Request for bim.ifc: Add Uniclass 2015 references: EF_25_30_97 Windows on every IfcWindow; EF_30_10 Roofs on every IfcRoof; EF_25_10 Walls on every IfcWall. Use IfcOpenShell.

First a look at what the model holds.

```python
import ifcopenshell

model = ifcopenshell.open("bim.ifc")
print(model.schema)
print("classifications:", [c.Name for c in model.by_type("IfcClassification")])
for ifc_class in ("IfcDoor", "IfcRoof", "IfcStair", "IfcWall", "IfcWindow"):
    print(ifc_class, len(model.by_type(ifc_class)))
```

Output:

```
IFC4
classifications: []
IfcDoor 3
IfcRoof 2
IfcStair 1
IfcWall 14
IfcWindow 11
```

```python
import ifcopenshell
import ifcopenshell.api.classification

model = ifcopenshell.open("bim.ifc")

system = ifcopenshell.api.classification.add_classification(model, classification="Uniclass 2015")

codes = {
    "IfcWindow": ("EF_25_30_97", "Windows"),
    "IfcRoof": ("EF_30_10", "Roofs"),
    "IfcWall": ("EF_25_10", "Walls"),
}
for ifc_class, (code, name) in codes.items():
    products = model.by_type(ifc_class)
    ifcopenshell.api.classification.add_reference(
        model, products=products, classification=system, identification=code, name=name
    )
    print(code, len(products))

model.write("bim_rev.ifc")
```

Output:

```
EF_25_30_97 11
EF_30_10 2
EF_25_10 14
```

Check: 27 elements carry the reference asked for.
